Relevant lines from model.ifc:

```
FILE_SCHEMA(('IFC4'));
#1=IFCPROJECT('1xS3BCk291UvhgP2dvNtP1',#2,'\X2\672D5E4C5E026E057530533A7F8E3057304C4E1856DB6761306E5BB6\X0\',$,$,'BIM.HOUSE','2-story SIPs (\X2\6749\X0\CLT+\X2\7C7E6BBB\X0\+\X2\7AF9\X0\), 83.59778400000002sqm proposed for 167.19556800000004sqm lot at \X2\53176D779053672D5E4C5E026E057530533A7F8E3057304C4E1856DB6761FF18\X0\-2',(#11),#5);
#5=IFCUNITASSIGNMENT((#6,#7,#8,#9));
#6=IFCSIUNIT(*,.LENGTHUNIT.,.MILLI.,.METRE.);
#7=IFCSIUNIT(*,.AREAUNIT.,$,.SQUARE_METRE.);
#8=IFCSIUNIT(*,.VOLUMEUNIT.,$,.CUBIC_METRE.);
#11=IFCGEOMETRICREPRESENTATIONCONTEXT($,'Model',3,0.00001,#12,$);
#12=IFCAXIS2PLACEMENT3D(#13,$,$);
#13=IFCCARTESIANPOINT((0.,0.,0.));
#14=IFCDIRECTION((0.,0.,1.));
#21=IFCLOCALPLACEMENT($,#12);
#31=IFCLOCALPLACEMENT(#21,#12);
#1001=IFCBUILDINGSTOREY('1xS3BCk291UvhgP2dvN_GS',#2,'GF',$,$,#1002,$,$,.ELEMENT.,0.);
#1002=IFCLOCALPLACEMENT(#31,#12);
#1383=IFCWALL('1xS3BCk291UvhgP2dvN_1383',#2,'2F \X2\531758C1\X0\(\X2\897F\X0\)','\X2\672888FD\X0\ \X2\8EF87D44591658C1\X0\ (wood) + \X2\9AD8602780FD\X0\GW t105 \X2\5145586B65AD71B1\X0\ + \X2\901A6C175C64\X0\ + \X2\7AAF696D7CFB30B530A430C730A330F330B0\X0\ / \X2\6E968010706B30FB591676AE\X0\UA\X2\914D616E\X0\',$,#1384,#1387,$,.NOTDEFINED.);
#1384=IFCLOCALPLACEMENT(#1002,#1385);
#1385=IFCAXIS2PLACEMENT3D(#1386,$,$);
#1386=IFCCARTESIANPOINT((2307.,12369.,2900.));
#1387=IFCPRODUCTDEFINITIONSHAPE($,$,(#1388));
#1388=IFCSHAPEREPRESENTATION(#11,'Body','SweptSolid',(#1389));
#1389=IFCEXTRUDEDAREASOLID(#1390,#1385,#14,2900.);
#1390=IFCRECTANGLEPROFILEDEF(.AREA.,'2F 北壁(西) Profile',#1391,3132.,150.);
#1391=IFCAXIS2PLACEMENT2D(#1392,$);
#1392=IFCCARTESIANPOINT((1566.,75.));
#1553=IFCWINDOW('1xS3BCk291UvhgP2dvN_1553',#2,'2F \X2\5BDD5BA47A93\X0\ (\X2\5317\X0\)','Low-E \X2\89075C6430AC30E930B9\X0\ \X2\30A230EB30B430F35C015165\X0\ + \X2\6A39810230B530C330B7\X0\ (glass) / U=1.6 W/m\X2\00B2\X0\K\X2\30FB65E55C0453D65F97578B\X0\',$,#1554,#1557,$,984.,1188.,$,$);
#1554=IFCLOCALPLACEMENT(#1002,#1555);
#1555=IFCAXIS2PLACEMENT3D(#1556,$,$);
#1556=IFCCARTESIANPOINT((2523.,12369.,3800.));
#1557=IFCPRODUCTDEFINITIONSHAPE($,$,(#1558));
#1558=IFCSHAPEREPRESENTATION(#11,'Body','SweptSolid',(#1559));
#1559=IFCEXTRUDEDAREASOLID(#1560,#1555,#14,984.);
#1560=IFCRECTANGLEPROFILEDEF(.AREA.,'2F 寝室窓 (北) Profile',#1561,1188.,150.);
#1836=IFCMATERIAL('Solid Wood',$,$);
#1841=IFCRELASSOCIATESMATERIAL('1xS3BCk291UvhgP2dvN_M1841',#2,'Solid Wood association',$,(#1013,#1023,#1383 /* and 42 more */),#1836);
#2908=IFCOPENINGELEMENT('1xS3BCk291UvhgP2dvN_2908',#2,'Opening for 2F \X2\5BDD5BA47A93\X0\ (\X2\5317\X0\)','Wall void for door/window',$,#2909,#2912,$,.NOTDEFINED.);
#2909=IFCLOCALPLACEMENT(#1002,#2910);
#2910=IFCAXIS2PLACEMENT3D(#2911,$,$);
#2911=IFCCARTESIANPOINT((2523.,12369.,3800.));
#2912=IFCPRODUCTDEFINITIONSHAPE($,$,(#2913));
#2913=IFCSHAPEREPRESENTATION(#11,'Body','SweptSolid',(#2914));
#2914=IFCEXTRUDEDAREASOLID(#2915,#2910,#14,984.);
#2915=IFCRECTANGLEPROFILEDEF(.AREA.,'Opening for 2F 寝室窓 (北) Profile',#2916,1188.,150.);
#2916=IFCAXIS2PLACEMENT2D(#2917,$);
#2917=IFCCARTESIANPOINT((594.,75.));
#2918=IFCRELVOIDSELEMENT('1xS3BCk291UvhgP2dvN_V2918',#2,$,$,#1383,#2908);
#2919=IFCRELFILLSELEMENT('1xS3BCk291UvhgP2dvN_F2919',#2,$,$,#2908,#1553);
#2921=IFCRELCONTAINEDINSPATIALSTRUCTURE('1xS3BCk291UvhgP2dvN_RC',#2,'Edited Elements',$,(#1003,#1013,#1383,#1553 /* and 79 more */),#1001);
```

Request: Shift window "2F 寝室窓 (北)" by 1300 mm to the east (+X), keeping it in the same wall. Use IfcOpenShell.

```python
import ifcopenshell
import ifcopenshell.api.geometry
import ifcopenshell.util.placement

model = ifcopenshell.open("model.ifc")

window = model.by_id(1553)
opening = window.FillsVoids[0].RelatingOpeningElement
wall = opening.VoidsElements[0].RelatingBuildingElement

wall_matrix = ifcopenshell.util.placement.get_local_placement(wall.ObjectPlacement)
shift = wall_matrix[:3, 0] * 1300.0
before = ifcopenshell.util.placement.get_local_placement(window.ObjectPlacement)[:3, 3].copy()

# The window is not placed relative to its opening, so move both.
for product in (opening, window):
    matrix = ifcopenshell.util.placement.get_local_placement(product.ObjectPlacement)
    matrix[:3, 3] += shift
    ifcopenshell.api.geometry.edit_object_placement(model, product=product, matrix=matrix, is_si=False)

after = ifcopenshell.util.placement.get_local_placement(window.ObjectPlacement)[:3, 3]
print("window moved by", (after - before).round(3) + 0.0)

model.write("model_v2.ifc")
```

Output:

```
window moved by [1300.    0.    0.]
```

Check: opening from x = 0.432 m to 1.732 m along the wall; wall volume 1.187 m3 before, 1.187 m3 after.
